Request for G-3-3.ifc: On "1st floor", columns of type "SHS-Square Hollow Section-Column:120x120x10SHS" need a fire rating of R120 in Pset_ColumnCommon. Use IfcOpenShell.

First a look at what the model holds.

```python
import ifcopenshell
import ifcopenshell.util.element

model = ifcopenshell.open("G-3-3.ifc")
print(model.schema)
storey = next(s for s in model.by_type("IfcBuildingStorey") if s.Name == "1st floor")
columns = [e for e in ifcopenshell.util.element.get_decomposition(storey) if e.is_a("IfcColumn")]
seen = {}
for e in columns:
    element_type = ifcopenshell.util.element.get_type(e)
    key = (element_type.Name if element_type != e and element_type else None, ifcopenshell.util.element.get_pset(e, "Pset_ColumnCommon", "FireRating"))
    seen[key] = seen.get(key, 0) + 1
for (name, value), count in sorted(seen.items(), key=str):
    print(count, "x", name, "|", value)
```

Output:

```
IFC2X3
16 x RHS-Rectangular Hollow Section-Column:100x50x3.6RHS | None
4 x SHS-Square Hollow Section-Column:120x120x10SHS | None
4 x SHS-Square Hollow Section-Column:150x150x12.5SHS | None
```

```python
import ifcopenshell
import ifcopenshell.api.pset
import ifcopenshell.util.element

model = ifcopenshell.open("G-3-3.ifc")

storey = next(s for s in model.by_type("IfcBuildingStorey") if s.Name == "1st floor")
columns = [e for e in ifcopenshell.util.element.get_decomposition(storey) if e.is_a("IfcColumn")]

count = 0
for e in columns:
    element_type = ifcopenshell.util.element.get_type(e)
    if element_type in (None, e) or element_type.Name != "SHS-Square Hollow Section-Column:120x120x10SHS":
        continue
    # add_pset returns the element's existing set when there is one.
    pset = ifcopenshell.api.pset.add_pset(model, product=e, name="Pset_ColumnCommon")
    ifcopenshell.api.pset.edit_pset(model, pset=pset, properties={"FireRating": "R120"})
    count += 1

print(count, "columns updated")

model.write("G-3-3_rev.ifc")
```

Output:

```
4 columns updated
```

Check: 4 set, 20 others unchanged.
